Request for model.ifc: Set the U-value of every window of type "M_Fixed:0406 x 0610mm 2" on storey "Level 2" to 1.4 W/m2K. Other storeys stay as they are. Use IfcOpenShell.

First a look at what the model holds.

```python
import ifcopenshell
import ifcopenshell.util.element

model = ifcopenshell.open("model.ifc")
print(model.schema)
storey = next(s for s in model.by_type("IfcBuildingStorey") if s.Name == "Level 2")
windows = [e for e in ifcopenshell.util.element.get_decomposition(storey) if e.is_a("IfcWindow")]
seen = {}
for e in windows:
    element_type = ifcopenshell.util.element.get_type(e)
    key = (element_type.Name if element_type != e and element_type else None, ifcopenshell.util.element.get_pset(e, "Pset_WindowCommon", "ThermalTransmittance"))
    seen[key] = seen.get(key, 0) + 1
for (name, value), count in sorted(seen.items(), key=str):
    print(count, "x", name, "|", value)
```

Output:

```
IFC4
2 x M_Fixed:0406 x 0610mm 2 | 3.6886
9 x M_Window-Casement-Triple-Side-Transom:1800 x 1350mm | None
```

```python
import ifcopenshell
import ifcopenshell.api.pset
import ifcopenshell.util.element

model = ifcopenshell.open("model.ifc")

storey = next(s for s in model.by_type("IfcBuildingStorey") if s.Name == "Level 2")
windows = [e for e in ifcopenshell.util.element.get_decomposition(storey) if e.is_a("IfcWindow")]

count = 0
for e in windows:
    element_type = ifcopenshell.util.element.get_type(e)
    if element_type in (None, e) or element_type.Name != "M_Fixed:0406 x 0610mm 2":
        continue
    # add_pset returns the element's existing set when there is one.
    pset = ifcopenshell.api.pset.add_pset(model, product=e, name="Pset_WindowCommon")
    ifcopenshell.api.pset.edit_pset(model, pset=pset, properties={"ThermalTransmittance": 1.4})
    count += 1

print(count, "windows updated")

model.write("model_rev.ifc")
```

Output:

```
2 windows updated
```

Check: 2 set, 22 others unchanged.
